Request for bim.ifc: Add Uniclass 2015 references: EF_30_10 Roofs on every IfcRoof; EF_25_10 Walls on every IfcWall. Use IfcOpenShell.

First a look at what the model holds.

```python
import ifcopenshell

model = ifcopenshell.open("bim.ifc")
print(model.schema)
print("classifications:", [c.Name for c in model.by_type("IfcClassification")])
for ifc_class in ("IfcDoor", "IfcRoof", "IfcStair", "IfcWall", "IfcWindow"):
    print(ifc_class, len(model.by_type(ifc_class)))
```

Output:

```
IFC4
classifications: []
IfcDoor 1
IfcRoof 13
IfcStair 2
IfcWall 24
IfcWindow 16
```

```python
import ifcopenshell
import ifcopenshell.api.classification

model = ifcopenshell.open("bim.ifc")

system = ifcopenshell.api.classification.add_classification(model, classification="Uniclass 2015")

codes = {
    "IfcRoof": ("EF_30_10", "Roofs"),
    "IfcWall": ("EF_25_10", "Walls"),
}
for ifc_class, (code, name) in codes.items():
    products = model.by_type(ifc_class)
    ifcopenshell.api.classification.add_reference(
        model, products=products, classification=system, identification=code, name=name
    )
    print(code, len(products))

model.write("bim_edited.ifc")
```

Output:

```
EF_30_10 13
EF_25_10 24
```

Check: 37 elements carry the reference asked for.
